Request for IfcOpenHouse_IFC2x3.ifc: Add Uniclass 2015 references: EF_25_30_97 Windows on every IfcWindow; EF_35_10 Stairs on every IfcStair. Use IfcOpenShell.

First a look at what the model holds.

```python
import ifcopenshell

model = ifcopenshell.open("IfcOpenHouse_IFC2x3.ifc")
print(model.schema)
print("classifications:", [c.Name for c in model.by_type("IfcClassification")])
for ifc_class in ("IfcDoor", "IfcRoof", "IfcStair", "IfcWall", "IfcWindow"):
    print(ifc_class, len(model.by_type(ifc_class)))
```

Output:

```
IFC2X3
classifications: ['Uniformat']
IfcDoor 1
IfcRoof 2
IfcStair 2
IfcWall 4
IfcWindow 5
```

```python
import ifcopenshell
import ifcopenshell.api.classification

model = ifcopenshell.open("IfcOpenHouse_IFC2x3.ifc")

# IFC2X3 requires Source and Edition and has no link from the project to the system.
system = model.create_entity("IfcClassification", Source="NBS", Edition="2015", Name="Uniclass 2015")

codes = {
    "IfcWindow": ("EF_25_30_97", "Windows"),
    "IfcStair": ("EF_35_10", "Stairs"),
}
for ifc_class, (code, name) in codes.items():
    products = model.by_type(ifc_class)
    ifcopenshell.api.classification.add_reference(
        model, products=products, classification=system, identification=code, name=name
    )
    print(code, len(products))

model.write("IfcOpenHouse_IFC2x3_rev.ifc")
```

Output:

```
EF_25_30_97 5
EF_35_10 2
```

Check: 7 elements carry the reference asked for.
